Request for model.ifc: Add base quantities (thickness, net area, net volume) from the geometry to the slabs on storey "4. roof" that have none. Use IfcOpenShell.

First a look at what the model holds.

```python
import ifcopenshell
import ifcopenshell.util.element
import ifcopenshell.util.unit

model = ifcopenshell.open("model.ifc")
print(model.schema)
for unit_type in ("LENGTHUNIT", "AREAUNIT", "VOLUMEUNIT"):
    print(unit_type, ifcopenshell.util.unit.calculate_unit_scale(model, unit_type))
storey = next(s for s in model.by_type("IfcBuildingStorey") if s.Name == "4. roof")
slabs = [e for e in ifcopenshell.util.element.get_decomposition(storey) if e.is_a("IfcSlab")]
for e in sorted(slabs, key=lambda e: e.id()):
    print(e.id(), e.is_a(), e.Name, list(ifcopenshell.util.element.get_psets(e, qtos_only=True)), sep=" | ")
```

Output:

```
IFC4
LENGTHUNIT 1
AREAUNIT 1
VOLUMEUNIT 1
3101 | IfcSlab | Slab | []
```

```python
import ifcopenshell
import ifcopenshell.api.pset
import ifcopenshell.geom
import ifcopenshell.util.element
import ifcopenshell.util.shape
import ifcopenshell.util.unit

model = ifcopenshell.open("model.ifc")
unit_scale = ifcopenshell.util.unit.calculate_unit_scale(model)
area_scale = ifcopenshell.util.unit.calculate_unit_scale(model, "AREAUNIT")
volume_scale = ifcopenshell.util.unit.calculate_unit_scale(model, "VOLUMEUNIT")
settings = ifcopenshell.geom.settings()

storey = next(s for s in model.by_type("IfcBuildingStorey") if s.Name == "4. roof")
slabs = [e for e in ifcopenshell.util.element.get_decomposition(storey) if e.is_a("IfcSlab")]

for e in sorted(slabs, key=lambda e: e.id()):
    if ifcopenshell.util.element.get_psets(e, qtos_only=True, should_inherit=False):
        continue
    # Geometry comes back in metres, in the element's own axes.
    shape = ifcopenshell.geom.create_shape(settings, e)
    values = {
        "Width": ifcopenshell.util.shape.get_z(shape.geometry) / unit_scale,
        "NetArea": ifcopenshell.util.shape.get_footprint_area(shape.geometry) / area_scale,
        "NetVolume": ifcopenshell.util.shape.get_volume(shape.geometry) / volume_scale,
    }
    qto = ifcopenshell.api.pset.add_qto(model, product=e, name="Qto_SlabBaseQuantities")
    ifcopenshell.api.pset.edit_qto(model, qto=qto, properties=values)
    print(e.id(), {k: round(v, 3) for k, v in values.items()})

model.write("model_rev.ifc")
```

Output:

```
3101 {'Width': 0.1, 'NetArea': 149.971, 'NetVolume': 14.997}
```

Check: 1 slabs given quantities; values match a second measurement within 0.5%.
